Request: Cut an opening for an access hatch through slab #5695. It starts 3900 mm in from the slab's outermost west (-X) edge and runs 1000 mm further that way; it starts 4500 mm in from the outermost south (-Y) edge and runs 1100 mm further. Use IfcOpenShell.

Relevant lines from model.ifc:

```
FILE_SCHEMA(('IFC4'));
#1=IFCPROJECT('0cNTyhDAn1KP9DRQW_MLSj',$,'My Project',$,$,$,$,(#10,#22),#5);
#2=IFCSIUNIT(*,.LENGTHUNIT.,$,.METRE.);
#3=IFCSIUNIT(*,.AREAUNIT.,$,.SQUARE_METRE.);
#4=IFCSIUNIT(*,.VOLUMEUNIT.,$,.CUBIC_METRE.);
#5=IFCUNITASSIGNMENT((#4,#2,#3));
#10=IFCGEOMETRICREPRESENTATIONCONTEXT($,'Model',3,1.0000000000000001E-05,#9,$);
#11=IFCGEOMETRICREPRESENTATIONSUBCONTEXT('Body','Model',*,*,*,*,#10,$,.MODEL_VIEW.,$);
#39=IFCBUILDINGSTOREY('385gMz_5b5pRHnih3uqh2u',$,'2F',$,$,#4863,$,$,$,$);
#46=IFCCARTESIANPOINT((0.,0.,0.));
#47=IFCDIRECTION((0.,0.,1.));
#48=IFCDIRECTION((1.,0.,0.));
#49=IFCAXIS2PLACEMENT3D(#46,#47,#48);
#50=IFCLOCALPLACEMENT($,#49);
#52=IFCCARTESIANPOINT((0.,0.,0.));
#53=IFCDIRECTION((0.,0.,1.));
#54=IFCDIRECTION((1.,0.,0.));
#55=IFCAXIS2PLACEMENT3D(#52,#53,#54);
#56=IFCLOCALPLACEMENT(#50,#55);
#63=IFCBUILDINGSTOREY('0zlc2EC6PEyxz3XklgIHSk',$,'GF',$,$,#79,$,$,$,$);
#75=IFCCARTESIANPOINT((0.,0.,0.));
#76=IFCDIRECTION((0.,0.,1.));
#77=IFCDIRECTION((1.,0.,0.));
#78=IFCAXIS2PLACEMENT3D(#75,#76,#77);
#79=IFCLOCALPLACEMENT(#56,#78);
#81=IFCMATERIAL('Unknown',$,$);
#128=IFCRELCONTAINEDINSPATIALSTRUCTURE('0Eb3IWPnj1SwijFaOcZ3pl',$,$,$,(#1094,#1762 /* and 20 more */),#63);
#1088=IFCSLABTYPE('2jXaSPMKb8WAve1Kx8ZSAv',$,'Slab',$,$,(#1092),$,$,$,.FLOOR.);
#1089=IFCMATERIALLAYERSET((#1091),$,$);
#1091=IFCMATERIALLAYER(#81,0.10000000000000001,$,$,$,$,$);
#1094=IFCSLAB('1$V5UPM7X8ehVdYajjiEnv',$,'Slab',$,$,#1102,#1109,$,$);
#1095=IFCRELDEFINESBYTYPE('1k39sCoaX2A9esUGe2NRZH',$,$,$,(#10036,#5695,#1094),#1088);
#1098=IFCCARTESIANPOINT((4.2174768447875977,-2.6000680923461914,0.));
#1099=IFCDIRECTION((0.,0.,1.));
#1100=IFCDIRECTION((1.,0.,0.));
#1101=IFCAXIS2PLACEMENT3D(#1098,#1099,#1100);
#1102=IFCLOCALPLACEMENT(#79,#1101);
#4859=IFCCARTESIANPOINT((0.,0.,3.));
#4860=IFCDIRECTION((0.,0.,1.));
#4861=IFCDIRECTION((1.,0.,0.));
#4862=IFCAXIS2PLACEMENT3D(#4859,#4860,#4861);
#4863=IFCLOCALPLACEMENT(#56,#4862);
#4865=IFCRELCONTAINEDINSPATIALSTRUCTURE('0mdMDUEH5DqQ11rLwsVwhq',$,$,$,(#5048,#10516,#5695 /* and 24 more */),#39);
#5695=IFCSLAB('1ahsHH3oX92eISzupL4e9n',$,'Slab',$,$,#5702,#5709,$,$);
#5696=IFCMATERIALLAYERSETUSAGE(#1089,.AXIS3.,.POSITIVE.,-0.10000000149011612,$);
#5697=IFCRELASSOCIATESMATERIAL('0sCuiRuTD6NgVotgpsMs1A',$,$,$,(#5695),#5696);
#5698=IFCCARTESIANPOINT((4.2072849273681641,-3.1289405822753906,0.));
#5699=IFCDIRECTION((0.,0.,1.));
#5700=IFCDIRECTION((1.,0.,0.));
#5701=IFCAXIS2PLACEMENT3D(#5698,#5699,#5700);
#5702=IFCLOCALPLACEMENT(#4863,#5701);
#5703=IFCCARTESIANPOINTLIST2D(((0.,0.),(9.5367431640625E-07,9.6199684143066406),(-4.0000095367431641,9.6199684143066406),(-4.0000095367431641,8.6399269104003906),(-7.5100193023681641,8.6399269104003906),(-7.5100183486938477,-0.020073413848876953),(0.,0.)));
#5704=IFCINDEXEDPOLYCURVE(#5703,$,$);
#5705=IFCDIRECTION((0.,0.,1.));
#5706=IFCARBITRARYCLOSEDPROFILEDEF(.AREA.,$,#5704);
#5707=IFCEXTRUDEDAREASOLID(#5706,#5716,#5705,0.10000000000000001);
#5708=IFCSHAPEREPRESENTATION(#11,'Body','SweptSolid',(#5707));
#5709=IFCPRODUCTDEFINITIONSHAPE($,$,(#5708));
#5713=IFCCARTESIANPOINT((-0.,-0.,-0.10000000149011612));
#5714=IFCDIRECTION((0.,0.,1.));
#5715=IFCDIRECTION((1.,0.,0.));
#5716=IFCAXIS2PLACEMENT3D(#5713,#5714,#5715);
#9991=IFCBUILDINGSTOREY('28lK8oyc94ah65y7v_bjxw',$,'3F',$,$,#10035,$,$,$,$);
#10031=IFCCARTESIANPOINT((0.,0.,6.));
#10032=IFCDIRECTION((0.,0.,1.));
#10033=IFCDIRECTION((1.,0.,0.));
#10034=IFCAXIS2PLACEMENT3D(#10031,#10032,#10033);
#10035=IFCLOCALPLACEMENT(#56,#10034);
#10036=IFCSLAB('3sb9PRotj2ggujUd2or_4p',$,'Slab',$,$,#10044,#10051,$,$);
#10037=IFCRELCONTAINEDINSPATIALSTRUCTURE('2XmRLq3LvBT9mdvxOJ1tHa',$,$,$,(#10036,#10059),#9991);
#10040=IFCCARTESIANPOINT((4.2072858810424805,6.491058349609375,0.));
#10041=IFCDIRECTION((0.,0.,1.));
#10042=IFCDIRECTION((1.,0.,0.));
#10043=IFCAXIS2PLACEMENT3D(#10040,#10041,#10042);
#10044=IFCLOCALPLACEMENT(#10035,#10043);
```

```python
import numpy as np
import ifcopenshell
import ifcopenshell.api.feature
import ifcopenshell.api.geometry
import ifcopenshell.api.root
import ifcopenshell.geom
import ifcopenshell.util.placement
import ifcopenshell.util.representation
import ifcopenshell.util.shape
import ifcopenshell.util.unit

model = ifcopenshell.open("model.ifc")
unit_scale = ifcopenshell.util.unit.calculate_unit_scale(model)
settings = ifcopenshell.geom.settings()


def volume(element):
    """Net volume in cubic metres, openings subtracted."""
    shape = ifcopenshell.geom.create_shape(settings, element)
    return ifcopenshell.util.shape.get_volume(shape.geometry)


slab = model.by_guid("1ahsHH3oX92eISzupL4e9n")
before = volume(slab)

# Extent in the slab's own axes, in metres. The edges named are its -X and -Y sides.
slab_shape = ifcopenshell.geom.create_shape(settings, slab)
vertices = ifcopenshell.util.shape.get_vertices(slab_shape.geometry)
x_min, y_min, bottom = vertices.min(axis=0)
top = vertices[:, 2].max()

opening = ifcopenshell.api.root.create_entity(model, ifc_class="IfcOpeningElement", name="Access hatch opening", predefined_type="OPENING")
context = ifcopenshell.util.representation.get_context(model, "Model", "Body", "MODEL_VIEW")
width, depth = 1, 1.1
outline = [(0.0, 0.0), (width, 0.0), (width, depth), (0.0, depth), (0.0, 0.0)]
# Overshoot both faces by 50 mm so the cut is clean.
shape = ifcopenshell.api.geometry.add_slab_representation(
    model, context=context, depth=top - bottom + 0.1, polyline=outline
)
ifcopenshell.api.geometry.assign_representation(model, product=opening, representation=shape)

matrix = ifcopenshell.util.placement.get_local_placement(slab.ObjectPlacement)
matrix[:, 3] = matrix @ np.append(np.array([x_min + 3.9, y_min + 4.5, bottom - 0.05]) / unit_scale, 1.0)
ifcopenshell.api.geometry.edit_object_placement(model, product=opening, matrix=matrix, is_si=False)
ifcopenshell.api.feature.add_feature(model, feature=opening, element=slab)

after = volume(slab)

print(f"slab volume {before:.3f} -> {after:.3f} m3")

model.write("model_rev.ifc")
```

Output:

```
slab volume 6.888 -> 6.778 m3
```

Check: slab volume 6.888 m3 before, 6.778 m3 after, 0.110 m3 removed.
